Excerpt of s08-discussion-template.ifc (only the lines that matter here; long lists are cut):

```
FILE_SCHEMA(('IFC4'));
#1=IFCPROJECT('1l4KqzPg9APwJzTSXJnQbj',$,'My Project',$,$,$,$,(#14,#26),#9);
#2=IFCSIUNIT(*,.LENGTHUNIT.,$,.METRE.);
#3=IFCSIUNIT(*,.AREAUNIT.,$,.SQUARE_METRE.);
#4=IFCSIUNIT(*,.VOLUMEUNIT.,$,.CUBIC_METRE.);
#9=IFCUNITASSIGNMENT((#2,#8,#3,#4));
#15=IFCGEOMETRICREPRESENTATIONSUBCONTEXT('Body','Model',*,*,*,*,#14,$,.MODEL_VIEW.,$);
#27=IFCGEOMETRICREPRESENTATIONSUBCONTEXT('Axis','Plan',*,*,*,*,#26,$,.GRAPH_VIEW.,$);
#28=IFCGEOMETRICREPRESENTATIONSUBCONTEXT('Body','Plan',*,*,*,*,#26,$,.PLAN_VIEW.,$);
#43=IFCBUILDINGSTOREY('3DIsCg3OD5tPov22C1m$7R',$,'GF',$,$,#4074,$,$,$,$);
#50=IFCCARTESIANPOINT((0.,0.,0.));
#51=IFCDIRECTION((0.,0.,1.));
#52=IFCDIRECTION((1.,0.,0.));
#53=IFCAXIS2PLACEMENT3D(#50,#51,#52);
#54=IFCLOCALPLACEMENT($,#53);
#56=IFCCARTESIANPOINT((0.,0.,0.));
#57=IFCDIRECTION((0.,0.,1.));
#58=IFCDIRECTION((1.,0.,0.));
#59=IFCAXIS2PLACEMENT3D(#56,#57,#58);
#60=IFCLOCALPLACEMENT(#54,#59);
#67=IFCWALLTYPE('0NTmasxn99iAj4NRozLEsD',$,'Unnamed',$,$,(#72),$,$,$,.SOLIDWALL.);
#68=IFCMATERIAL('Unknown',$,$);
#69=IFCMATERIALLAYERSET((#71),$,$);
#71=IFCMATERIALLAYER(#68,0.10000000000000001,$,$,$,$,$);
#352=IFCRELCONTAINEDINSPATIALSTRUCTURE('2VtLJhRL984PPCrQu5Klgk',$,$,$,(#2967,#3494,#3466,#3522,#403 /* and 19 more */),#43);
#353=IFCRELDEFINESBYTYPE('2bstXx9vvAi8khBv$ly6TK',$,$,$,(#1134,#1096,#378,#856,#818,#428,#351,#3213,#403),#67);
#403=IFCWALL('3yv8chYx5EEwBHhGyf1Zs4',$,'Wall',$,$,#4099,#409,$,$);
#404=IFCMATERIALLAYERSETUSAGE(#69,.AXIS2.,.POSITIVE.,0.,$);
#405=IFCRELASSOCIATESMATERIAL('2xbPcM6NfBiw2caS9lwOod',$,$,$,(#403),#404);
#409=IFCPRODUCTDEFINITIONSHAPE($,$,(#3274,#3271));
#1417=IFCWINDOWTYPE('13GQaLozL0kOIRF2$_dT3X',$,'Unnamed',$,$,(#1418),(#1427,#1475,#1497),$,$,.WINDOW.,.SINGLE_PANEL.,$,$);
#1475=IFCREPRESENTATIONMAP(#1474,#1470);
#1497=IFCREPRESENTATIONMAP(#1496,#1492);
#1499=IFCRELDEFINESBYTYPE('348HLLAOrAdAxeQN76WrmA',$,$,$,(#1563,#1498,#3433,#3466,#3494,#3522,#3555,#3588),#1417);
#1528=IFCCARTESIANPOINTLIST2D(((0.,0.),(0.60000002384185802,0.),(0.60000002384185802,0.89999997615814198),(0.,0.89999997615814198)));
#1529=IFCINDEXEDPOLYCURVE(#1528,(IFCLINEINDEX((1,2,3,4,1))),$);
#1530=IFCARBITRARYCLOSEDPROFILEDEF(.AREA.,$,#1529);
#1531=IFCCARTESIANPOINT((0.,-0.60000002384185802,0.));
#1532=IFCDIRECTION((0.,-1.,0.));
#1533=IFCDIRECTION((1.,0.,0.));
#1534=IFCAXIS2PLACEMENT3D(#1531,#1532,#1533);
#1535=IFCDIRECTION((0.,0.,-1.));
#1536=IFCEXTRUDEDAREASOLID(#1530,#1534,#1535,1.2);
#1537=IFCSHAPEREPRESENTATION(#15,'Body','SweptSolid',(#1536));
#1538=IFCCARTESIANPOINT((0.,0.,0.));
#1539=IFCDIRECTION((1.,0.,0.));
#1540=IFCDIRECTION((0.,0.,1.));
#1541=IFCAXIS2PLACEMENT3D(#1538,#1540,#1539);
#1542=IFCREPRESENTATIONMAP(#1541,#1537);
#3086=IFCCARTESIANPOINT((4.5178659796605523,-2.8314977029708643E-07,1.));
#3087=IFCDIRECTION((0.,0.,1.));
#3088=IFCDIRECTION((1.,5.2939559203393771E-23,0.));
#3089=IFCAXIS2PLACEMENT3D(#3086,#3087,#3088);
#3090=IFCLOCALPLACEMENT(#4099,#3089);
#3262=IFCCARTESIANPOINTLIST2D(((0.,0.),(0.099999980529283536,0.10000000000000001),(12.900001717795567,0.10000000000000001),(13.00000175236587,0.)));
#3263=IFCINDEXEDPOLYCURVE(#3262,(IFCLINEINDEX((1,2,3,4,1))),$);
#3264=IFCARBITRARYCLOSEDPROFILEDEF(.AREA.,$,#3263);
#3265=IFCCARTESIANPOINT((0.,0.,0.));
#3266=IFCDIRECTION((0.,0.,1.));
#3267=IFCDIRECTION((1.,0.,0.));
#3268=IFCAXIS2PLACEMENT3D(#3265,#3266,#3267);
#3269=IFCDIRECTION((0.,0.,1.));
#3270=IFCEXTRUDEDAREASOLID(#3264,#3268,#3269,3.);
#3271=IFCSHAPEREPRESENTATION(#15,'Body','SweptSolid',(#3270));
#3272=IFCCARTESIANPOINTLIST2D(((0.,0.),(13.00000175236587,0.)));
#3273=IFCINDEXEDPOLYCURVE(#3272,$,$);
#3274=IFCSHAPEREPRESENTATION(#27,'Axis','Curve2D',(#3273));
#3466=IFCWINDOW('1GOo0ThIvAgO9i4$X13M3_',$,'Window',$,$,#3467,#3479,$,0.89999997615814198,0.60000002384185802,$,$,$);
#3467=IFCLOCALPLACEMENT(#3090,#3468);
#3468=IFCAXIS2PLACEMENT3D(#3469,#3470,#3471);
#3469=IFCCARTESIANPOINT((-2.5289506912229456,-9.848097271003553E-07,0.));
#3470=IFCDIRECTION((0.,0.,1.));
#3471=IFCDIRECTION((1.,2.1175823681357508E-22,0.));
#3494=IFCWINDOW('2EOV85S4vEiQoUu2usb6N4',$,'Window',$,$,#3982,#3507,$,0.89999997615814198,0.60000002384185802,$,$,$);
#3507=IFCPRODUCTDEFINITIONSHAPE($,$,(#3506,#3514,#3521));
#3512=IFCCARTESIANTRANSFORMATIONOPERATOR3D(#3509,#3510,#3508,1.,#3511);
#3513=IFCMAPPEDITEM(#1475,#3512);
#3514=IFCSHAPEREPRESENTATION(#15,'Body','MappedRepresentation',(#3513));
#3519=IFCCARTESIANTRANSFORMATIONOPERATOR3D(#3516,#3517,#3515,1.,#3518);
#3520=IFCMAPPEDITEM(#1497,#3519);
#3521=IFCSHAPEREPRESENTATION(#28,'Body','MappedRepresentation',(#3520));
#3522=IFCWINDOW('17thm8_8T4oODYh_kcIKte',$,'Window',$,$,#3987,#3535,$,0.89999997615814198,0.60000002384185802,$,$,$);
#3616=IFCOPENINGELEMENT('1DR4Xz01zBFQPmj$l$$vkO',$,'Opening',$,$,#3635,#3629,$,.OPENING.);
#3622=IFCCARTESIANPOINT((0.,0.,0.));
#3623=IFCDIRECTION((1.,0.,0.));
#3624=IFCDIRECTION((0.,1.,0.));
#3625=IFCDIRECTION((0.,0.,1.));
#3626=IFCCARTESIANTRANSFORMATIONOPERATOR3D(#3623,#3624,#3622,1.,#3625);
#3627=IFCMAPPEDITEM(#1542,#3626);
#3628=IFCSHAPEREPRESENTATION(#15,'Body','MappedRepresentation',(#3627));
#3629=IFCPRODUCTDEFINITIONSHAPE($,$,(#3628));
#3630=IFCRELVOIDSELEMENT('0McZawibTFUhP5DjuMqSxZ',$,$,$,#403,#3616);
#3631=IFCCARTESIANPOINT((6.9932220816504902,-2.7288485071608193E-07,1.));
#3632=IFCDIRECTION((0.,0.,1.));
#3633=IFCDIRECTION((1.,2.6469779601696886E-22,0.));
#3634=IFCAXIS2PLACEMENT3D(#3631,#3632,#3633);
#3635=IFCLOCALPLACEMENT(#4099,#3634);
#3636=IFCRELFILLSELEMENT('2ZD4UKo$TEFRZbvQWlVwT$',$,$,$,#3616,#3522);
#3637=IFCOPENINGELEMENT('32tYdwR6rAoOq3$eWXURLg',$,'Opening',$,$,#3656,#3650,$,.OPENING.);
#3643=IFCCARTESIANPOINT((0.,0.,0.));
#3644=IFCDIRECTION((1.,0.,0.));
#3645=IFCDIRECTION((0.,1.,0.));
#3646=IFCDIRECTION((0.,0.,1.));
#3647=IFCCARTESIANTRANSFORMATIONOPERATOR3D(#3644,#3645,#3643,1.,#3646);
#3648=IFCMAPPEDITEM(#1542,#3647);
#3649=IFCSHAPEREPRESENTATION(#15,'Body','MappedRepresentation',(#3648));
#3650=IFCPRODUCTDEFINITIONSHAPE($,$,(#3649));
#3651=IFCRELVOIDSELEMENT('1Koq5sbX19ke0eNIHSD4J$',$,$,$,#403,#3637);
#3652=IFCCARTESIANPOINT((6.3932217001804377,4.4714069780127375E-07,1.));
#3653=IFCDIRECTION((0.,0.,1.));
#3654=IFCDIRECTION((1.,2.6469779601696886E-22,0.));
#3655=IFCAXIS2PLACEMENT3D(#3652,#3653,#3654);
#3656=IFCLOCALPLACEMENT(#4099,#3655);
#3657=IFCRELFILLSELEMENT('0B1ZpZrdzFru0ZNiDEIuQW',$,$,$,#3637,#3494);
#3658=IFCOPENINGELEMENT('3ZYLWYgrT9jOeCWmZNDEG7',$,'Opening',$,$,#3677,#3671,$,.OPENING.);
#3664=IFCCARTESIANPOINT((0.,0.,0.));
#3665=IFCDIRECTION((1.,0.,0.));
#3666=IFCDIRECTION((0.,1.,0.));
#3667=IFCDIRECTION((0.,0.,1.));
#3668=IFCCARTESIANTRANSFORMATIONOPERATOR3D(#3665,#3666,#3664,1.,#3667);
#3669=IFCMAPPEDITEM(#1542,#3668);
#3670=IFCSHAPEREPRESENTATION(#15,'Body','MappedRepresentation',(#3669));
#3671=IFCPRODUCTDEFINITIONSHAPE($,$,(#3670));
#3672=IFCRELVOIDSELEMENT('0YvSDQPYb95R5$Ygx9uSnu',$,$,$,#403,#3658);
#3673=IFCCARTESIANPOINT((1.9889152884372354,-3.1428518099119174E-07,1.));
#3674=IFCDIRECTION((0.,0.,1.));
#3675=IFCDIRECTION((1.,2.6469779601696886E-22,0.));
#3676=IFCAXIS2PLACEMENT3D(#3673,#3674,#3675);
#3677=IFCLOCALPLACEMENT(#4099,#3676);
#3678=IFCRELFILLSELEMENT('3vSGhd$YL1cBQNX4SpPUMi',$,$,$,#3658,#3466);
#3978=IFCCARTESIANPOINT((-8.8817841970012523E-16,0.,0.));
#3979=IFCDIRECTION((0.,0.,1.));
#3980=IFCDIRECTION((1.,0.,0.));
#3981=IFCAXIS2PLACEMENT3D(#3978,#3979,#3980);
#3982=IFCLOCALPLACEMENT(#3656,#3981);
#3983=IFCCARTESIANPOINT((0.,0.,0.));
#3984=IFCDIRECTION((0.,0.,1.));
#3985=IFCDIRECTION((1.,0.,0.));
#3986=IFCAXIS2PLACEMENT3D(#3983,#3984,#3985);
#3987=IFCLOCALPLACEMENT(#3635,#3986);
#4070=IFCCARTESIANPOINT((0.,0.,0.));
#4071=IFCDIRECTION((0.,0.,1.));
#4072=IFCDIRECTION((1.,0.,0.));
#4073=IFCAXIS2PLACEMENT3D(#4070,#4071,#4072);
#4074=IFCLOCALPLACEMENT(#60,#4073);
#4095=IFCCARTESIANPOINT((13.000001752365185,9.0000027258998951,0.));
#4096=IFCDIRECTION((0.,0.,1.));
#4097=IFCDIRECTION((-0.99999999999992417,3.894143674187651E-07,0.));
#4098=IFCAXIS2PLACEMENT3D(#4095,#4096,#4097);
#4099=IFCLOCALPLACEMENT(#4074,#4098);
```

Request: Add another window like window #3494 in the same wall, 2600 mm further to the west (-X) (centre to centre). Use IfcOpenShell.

```python
import ifcopenshell
import ifcopenshell.api.feature
import ifcopenshell.api.geometry
import ifcopenshell.api.root
import ifcopenshell.geom
import ifcopenshell.util.element
import ifcopenshell.util.placement
import ifcopenshell.util.shape

model = ifcopenshell.open("s08-discussion-template.ifc")
settings = ifcopenshell.geom.settings()


def volume(element):
    """Net volume in cubic metres, openings subtracted."""
    shape = ifcopenshell.geom.create_shape(settings, element)
    return ifcopenshell.util.shape.get_volume(shape.geometry)


window = model.by_guid("2EOV85S4vEiQoUu2usb6N4")
opening = window.FillsVoids[0].RelatingOpeningElement
wall = opening.VoidsElements[0].RelatingBuildingElement
before = volume(wall)
shift = ifcopenshell.util.placement.get_local_placement(wall.ObjectPlacement)[:3, 0] * 2.6

# copy_class copies the void relationship, type, container and properties, but no geometry.
new_opening = ifcopenshell.api.root.copy_class(model, product=opening)
new_opening.Representation = ifcopenshell.util.element.copy_deep(
    model, opening.Representation, exclude=["IfcGeometricRepresentationContext", "IfcRepresentationMap"]
)
new_window = ifcopenshell.api.root.copy_class(model, product=window)
new_window.Representation = ifcopenshell.util.element.copy_deep(
    model, window.Representation, exclude=["IfcGeometricRepresentationContext", "IfcRepresentationMap"]
)
ifcopenshell.api.feature.add_filling(model, opening=new_opening, element=new_window)

for old, new in ((opening, new_opening), (window, new_window)):
    matrix = ifcopenshell.util.placement.get_local_placement(old.ObjectPlacement)
    matrix[:3, 3] += shift
    ifcopenshell.api.geometry.edit_object_placement(model, product=new, matrix=matrix, is_si=False)

after = volume(wall)

print(f"wall volume {before:.3f} -> {after:.3f} m3")

model.write("s08-discussion-template_v2.ifc")
```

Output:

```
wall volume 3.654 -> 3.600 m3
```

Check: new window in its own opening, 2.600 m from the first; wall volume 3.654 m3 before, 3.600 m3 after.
